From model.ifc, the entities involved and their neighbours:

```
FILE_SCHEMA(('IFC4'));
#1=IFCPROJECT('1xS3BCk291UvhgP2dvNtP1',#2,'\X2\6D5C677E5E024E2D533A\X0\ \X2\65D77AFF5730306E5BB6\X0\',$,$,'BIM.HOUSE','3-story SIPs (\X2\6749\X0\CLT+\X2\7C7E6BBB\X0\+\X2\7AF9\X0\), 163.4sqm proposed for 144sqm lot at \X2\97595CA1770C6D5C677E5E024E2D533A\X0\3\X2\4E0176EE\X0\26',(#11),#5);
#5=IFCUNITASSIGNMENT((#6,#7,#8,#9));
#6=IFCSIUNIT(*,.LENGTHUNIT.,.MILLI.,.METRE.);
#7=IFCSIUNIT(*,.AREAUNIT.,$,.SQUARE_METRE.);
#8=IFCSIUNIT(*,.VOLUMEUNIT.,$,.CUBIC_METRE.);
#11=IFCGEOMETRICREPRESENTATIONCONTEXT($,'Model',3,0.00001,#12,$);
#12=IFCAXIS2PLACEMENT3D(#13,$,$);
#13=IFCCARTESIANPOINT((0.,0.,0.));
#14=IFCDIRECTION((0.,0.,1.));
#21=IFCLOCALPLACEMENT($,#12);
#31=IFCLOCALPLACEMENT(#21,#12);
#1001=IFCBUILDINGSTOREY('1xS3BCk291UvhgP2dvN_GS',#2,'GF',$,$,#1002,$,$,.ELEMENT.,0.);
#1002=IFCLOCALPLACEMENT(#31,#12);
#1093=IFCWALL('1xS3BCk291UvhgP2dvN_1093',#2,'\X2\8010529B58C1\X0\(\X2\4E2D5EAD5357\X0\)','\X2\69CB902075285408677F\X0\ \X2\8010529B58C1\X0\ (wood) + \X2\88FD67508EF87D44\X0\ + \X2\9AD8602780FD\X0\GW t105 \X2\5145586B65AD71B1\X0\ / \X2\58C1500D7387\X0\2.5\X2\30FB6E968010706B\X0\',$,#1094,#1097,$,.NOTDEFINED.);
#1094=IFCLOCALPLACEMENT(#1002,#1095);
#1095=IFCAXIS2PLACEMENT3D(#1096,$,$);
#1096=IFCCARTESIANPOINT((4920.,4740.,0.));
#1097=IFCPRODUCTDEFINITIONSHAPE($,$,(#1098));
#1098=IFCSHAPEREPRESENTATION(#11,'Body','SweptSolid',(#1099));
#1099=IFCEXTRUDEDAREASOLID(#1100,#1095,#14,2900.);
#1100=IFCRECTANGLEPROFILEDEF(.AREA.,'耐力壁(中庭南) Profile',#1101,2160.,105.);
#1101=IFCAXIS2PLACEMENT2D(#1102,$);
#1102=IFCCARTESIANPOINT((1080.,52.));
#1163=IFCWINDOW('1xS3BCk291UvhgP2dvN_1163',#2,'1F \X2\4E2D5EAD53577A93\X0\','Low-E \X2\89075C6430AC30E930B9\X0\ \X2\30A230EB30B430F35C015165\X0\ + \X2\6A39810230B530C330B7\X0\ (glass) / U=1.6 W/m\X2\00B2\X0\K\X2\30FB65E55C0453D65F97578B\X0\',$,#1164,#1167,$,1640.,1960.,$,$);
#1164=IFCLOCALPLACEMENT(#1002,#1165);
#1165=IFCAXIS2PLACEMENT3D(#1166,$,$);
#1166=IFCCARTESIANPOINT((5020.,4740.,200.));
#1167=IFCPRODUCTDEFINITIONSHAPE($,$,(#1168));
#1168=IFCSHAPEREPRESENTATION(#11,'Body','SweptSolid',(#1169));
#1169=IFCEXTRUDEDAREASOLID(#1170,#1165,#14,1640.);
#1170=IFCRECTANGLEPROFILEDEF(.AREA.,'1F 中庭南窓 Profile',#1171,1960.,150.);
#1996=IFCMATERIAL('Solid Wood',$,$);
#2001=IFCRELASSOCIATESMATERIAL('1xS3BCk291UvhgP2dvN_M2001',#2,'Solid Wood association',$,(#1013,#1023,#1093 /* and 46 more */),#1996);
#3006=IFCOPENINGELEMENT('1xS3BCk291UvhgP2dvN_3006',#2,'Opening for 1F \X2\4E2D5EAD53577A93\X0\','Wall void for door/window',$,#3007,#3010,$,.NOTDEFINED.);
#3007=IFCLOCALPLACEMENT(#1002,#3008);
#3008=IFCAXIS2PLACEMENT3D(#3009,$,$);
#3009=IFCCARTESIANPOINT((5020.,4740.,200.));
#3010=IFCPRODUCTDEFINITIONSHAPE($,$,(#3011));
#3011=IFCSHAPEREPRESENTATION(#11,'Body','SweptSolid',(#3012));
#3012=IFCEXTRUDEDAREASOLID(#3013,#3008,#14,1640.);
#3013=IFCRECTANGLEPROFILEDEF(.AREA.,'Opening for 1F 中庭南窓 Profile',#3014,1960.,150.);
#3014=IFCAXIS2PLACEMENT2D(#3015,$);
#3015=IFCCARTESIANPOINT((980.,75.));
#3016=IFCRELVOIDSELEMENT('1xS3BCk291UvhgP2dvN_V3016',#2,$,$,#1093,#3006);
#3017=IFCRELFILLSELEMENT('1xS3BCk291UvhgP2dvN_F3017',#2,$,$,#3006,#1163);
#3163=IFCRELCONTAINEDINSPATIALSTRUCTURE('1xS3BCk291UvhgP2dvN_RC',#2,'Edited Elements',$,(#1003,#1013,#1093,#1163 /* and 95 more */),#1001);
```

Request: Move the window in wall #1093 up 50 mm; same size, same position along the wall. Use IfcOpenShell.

```python
import numpy as np
import ifcopenshell
import ifcopenshell.api.geometry
import ifcopenshell.util.placement
import ifcopenshell.util.unit

model = ifcopenshell.open("model.ifc")
unit_scale = ifcopenshell.util.unit.calculate_unit_scale(model)

window = model.by_guid("1xS3BCk291UvhgP2dvN_1163")
opening = window.FillsVoids[0].RelatingOpeningElement
dz = 0.05 / unit_scale

shift = np.array([0.0, 0.0, dz])
# The window is not placed relative to its opening, so move both.
for product in (opening, window):
    matrix = ifcopenshell.util.placement.get_local_placement(product.ObjectPlacement)
    matrix[:3, 3] += shift
    ifcopenshell.api.geometry.edit_object_placement(model, product=product, matrix=matrix, is_si=False)

print(f"moved by {dz * unit_scale:+.3f} m")

model.write("model-out.ifc")
```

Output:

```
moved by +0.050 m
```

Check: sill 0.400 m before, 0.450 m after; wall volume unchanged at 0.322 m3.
